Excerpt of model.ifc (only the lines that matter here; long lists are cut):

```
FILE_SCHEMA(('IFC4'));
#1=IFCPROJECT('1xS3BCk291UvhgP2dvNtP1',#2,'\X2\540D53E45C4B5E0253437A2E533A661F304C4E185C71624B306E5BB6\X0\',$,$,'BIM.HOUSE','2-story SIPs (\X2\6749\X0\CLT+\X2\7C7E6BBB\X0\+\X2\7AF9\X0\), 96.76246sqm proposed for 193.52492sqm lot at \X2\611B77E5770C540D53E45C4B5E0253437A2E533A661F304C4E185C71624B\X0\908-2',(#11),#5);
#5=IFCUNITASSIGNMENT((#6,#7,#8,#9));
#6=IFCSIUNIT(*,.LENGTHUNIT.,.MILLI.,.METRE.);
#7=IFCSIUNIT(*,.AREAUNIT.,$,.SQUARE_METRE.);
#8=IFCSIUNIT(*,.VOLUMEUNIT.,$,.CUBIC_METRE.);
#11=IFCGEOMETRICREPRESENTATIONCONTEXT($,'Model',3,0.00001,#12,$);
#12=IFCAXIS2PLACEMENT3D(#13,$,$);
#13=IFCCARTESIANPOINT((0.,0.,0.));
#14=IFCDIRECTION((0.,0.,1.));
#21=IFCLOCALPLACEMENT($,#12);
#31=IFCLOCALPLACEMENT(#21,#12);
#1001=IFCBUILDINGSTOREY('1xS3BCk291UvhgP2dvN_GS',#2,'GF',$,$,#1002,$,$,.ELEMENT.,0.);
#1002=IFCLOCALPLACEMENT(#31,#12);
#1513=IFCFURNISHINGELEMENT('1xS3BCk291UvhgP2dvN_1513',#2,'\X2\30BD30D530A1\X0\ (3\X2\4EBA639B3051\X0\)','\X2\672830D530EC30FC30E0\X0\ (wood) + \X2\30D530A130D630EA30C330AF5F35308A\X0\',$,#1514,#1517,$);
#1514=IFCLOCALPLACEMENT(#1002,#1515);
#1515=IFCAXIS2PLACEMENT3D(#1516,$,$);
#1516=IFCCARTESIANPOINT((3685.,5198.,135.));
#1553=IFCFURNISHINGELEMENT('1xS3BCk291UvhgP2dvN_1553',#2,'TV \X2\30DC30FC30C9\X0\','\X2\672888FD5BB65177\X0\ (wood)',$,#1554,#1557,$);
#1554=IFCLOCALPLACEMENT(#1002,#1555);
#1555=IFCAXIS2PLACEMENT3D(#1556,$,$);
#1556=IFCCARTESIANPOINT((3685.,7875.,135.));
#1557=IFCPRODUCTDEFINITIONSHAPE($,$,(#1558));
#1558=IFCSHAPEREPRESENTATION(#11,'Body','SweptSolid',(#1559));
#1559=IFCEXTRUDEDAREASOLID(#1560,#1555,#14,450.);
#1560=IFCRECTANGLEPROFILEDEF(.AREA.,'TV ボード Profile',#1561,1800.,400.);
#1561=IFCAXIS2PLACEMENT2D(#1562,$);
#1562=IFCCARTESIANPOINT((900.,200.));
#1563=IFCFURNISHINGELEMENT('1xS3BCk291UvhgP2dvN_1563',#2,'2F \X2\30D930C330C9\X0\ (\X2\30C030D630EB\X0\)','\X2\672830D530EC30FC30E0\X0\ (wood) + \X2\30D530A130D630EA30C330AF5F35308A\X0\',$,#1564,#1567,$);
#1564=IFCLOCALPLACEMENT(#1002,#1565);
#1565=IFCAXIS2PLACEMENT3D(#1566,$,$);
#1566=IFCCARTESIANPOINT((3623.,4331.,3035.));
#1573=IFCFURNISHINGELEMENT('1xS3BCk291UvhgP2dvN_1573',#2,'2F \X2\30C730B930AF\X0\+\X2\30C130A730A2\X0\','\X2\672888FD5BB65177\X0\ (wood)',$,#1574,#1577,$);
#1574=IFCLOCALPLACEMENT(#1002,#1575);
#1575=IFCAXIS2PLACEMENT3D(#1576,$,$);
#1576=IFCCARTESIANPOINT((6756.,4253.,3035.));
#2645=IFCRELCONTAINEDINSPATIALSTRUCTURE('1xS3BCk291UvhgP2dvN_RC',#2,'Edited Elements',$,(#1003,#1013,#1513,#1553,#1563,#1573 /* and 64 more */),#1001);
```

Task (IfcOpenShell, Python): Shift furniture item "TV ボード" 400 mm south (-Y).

```python
import ifcopenshell
import ifcopenshell.api.geometry
import ifcopenshell.util.placement

model = ifcopenshell.open("model.ifc")

item = model.by_guid("1xS3BCk291UvhgP2dvN_1553")
matrix = ifcopenshell.util.placement.get_local_placement(item.ObjectPlacement)
matrix[1, 3] -= 400.0
ifcopenshell.api.geometry.edit_object_placement(model, product=item, matrix=matrix, is_si=False)

print(ifcopenshell.util.placement.get_local_placement(item.ObjectPlacement).round(3) + 0.0)

model.write("model_updated.ifc")
```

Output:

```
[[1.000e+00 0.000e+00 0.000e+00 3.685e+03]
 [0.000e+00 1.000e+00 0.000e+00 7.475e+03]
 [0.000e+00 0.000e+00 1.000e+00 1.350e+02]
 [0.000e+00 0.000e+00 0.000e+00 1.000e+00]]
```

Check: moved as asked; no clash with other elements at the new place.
